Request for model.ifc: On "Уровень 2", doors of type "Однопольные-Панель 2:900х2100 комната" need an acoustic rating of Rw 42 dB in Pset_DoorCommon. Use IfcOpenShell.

First a look at what the model holds.

```python
import ifcopenshell
import ifcopenshell.util.element

model = ifcopenshell.open("model.ifc")
print(model.schema)
storey = next(s for s in model.by_type("IfcBuildingStorey") if s.Name == "Уровень 2")
doors = [e for e in ifcopenshell.util.element.get_decomposition(storey) if e.is_a("IfcDoor")]
seen = {}
for e in doors:
    element_type = ifcopenshell.util.element.get_type(e)
    key = (element_type.Name if element_type != e and element_type else None, ifcopenshell.util.element.get_pset(e, "Pset_DoorCommon", "AcousticRating"))
    seen[key] = seen.get(key, 0) + 1
for (name, value), count in sorted(seen.items(), key=str):
    print(count, "x", name, "|", value)
```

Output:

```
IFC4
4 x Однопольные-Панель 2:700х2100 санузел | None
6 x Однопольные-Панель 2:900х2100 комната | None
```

```python
import ifcopenshell
import ifcopenshell.api.pset
import ifcopenshell.util.element

model = ifcopenshell.open("model.ifc")

storey = next(s for s in model.by_type("IfcBuildingStorey") if s.Name == "Уровень 2")
doors = [e for e in ifcopenshell.util.element.get_decomposition(storey) if e.is_a("IfcDoor")]

count = 0
for e in doors:
    element_type = ifcopenshell.util.element.get_type(e)
    if element_type in (None, e) or element_type.Name != "Однопольные-Панель 2:900х2100 комната":
        continue
    # add_pset returns the element's existing set when there is one.
    pset = ifcopenshell.api.pset.add_pset(model, product=e, name="Pset_DoorCommon")
    ifcopenshell.api.pset.edit_pset(model, pset=pset, properties={"AcousticRating": "Rw 42 dB"})
    count += 1

print(count, "doors updated")

model.write("model_edited.ifc")
```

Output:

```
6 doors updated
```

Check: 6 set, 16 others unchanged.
